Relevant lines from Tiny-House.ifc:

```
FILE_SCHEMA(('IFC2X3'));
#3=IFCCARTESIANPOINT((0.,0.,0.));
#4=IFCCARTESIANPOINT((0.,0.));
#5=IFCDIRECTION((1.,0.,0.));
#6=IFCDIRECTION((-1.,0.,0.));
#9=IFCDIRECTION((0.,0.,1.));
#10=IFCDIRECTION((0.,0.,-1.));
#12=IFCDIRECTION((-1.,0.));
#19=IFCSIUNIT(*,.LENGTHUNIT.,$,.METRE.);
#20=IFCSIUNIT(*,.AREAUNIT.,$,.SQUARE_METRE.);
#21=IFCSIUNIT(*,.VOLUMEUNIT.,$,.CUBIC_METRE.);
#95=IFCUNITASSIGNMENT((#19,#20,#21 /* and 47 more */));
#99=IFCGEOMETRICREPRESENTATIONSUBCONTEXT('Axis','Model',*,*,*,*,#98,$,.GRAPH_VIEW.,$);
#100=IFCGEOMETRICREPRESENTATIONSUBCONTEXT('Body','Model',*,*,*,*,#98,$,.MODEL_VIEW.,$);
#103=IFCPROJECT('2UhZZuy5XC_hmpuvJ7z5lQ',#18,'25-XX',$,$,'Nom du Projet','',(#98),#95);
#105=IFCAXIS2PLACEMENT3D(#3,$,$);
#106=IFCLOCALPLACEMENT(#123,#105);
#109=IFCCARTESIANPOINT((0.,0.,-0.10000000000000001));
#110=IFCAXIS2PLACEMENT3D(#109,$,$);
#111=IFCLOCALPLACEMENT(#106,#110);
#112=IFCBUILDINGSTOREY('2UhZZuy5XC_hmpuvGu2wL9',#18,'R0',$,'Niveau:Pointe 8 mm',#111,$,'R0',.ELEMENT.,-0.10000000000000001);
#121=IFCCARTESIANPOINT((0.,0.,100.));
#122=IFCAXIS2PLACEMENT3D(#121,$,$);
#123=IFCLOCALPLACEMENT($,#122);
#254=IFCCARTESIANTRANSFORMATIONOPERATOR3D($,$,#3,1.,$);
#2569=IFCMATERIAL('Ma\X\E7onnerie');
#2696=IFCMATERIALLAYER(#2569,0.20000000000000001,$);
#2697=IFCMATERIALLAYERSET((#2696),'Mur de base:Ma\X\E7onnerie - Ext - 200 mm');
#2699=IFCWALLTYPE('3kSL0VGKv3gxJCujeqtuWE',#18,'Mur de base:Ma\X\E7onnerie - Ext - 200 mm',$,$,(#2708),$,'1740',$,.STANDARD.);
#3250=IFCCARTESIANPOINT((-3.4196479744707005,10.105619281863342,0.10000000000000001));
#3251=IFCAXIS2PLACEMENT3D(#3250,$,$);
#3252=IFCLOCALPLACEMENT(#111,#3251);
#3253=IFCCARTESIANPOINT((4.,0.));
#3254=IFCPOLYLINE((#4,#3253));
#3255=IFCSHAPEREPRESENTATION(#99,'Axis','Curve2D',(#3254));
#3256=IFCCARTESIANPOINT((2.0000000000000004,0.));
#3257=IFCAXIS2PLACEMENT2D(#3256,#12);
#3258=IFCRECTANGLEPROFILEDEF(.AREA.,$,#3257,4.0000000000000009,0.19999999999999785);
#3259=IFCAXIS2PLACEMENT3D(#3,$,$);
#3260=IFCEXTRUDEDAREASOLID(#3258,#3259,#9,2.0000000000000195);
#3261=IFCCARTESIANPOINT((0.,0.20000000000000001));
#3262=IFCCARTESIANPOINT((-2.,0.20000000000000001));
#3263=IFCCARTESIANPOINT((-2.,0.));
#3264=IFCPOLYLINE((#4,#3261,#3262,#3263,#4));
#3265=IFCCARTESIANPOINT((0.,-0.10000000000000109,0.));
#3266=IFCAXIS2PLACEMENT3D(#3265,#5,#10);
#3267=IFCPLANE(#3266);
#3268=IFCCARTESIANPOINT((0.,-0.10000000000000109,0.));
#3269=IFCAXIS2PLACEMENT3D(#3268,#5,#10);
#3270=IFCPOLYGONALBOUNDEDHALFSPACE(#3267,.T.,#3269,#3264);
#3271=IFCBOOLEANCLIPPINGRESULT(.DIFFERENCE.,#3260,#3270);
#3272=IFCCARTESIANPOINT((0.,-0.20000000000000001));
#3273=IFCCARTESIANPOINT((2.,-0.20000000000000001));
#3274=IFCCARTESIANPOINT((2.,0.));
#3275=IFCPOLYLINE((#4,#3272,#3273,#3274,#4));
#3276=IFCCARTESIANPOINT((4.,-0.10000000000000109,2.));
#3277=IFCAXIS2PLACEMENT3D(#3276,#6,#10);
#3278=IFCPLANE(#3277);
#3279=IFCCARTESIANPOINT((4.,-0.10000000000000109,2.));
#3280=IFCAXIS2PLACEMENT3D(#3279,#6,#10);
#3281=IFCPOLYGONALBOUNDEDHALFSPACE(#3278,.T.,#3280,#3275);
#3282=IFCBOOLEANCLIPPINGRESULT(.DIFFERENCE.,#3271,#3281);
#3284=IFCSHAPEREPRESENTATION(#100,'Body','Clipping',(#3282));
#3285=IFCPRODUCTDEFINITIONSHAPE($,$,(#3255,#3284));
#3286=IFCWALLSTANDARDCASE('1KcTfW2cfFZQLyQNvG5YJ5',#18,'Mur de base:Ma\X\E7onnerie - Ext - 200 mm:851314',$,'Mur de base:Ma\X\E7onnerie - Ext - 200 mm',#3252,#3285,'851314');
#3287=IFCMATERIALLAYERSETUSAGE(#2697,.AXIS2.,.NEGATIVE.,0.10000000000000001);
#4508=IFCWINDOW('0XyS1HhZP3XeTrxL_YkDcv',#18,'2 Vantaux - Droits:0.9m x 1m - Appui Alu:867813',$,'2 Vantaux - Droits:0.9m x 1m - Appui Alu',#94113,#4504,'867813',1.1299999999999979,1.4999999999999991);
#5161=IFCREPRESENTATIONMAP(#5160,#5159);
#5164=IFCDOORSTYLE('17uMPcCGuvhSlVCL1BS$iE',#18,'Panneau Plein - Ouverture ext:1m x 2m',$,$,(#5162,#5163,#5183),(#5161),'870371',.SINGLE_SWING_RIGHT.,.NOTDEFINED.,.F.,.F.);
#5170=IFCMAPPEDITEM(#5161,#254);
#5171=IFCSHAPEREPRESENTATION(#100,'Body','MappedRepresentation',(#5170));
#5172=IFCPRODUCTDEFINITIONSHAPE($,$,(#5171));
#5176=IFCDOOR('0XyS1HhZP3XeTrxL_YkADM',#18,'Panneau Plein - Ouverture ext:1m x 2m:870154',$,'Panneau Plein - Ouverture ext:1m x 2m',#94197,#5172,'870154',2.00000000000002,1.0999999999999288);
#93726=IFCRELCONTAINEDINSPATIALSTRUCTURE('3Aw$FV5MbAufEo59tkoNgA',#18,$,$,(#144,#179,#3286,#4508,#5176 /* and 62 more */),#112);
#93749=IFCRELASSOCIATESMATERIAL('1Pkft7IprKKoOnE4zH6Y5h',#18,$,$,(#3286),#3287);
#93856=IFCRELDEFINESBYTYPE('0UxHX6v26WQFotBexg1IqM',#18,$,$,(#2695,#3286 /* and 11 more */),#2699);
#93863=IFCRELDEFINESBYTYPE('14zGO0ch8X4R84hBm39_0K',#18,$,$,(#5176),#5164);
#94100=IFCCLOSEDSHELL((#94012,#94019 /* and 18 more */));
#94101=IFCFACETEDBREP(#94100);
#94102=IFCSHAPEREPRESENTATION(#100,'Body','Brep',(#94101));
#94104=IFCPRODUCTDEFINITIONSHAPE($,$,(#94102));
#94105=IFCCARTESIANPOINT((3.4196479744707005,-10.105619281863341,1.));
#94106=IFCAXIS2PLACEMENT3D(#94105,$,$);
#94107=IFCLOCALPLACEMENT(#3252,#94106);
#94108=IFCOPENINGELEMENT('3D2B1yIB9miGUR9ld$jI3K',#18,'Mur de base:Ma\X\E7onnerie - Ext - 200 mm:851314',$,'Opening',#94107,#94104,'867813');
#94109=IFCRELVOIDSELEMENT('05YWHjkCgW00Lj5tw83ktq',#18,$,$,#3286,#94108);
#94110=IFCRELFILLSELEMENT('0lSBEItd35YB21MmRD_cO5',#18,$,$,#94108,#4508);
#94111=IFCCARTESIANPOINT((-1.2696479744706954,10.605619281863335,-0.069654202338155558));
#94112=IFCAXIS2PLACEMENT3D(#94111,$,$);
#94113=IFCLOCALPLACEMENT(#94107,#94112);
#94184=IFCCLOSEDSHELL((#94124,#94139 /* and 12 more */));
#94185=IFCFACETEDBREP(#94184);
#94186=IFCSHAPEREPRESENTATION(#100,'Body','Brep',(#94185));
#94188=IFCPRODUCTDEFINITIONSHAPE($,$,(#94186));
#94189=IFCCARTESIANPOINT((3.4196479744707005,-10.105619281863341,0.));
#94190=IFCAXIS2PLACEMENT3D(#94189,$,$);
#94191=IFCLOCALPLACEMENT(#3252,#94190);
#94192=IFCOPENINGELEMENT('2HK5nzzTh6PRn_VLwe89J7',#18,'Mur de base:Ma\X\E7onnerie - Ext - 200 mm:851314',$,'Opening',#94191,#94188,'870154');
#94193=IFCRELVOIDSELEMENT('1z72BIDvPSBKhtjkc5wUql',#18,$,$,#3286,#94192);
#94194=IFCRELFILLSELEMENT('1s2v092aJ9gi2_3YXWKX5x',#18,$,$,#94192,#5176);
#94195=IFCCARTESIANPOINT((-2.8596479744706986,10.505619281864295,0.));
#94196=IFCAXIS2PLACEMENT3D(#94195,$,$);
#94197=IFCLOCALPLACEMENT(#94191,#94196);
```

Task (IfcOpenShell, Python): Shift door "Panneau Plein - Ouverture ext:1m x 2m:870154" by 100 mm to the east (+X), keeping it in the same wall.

```python
import ifcopenshell
import ifcopenshell.api.geometry
import ifcopenshell.util.placement

model = ifcopenshell.open("Tiny-House.ifc")

door = model.by_guid("0XyS1HhZP3XeTrxL_YkADM")
opening = door.FillsVoids[0].RelatingOpeningElement
wall = opening.VoidsElements[0].RelatingBuildingElement

wall_matrix = ifcopenshell.util.placement.get_local_placement(wall.ObjectPlacement)
shift = wall_matrix[:3, 0] * 0.1
before = ifcopenshell.util.placement.get_local_placement(door.ObjectPlacement)[:3, 3].copy()

# The door is placed relative to its opening, so it follows when the opening moves.
matrix = ifcopenshell.util.placement.get_local_placement(opening.ObjectPlacement)
matrix[:3, 3] += shift
ifcopenshell.api.geometry.edit_object_placement(
    model, product=opening, matrix=matrix, is_si=False, should_transform_children=True
)

after = ifcopenshell.util.placement.get_local_placement(door.ObjectPlacement)[:3, 3]
print("door moved by", (after - before).round(3) + 0.0)

model.write("Tiny-House_updated.ifc")
```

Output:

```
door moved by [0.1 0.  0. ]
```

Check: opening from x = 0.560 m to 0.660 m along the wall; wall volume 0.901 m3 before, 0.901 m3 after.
